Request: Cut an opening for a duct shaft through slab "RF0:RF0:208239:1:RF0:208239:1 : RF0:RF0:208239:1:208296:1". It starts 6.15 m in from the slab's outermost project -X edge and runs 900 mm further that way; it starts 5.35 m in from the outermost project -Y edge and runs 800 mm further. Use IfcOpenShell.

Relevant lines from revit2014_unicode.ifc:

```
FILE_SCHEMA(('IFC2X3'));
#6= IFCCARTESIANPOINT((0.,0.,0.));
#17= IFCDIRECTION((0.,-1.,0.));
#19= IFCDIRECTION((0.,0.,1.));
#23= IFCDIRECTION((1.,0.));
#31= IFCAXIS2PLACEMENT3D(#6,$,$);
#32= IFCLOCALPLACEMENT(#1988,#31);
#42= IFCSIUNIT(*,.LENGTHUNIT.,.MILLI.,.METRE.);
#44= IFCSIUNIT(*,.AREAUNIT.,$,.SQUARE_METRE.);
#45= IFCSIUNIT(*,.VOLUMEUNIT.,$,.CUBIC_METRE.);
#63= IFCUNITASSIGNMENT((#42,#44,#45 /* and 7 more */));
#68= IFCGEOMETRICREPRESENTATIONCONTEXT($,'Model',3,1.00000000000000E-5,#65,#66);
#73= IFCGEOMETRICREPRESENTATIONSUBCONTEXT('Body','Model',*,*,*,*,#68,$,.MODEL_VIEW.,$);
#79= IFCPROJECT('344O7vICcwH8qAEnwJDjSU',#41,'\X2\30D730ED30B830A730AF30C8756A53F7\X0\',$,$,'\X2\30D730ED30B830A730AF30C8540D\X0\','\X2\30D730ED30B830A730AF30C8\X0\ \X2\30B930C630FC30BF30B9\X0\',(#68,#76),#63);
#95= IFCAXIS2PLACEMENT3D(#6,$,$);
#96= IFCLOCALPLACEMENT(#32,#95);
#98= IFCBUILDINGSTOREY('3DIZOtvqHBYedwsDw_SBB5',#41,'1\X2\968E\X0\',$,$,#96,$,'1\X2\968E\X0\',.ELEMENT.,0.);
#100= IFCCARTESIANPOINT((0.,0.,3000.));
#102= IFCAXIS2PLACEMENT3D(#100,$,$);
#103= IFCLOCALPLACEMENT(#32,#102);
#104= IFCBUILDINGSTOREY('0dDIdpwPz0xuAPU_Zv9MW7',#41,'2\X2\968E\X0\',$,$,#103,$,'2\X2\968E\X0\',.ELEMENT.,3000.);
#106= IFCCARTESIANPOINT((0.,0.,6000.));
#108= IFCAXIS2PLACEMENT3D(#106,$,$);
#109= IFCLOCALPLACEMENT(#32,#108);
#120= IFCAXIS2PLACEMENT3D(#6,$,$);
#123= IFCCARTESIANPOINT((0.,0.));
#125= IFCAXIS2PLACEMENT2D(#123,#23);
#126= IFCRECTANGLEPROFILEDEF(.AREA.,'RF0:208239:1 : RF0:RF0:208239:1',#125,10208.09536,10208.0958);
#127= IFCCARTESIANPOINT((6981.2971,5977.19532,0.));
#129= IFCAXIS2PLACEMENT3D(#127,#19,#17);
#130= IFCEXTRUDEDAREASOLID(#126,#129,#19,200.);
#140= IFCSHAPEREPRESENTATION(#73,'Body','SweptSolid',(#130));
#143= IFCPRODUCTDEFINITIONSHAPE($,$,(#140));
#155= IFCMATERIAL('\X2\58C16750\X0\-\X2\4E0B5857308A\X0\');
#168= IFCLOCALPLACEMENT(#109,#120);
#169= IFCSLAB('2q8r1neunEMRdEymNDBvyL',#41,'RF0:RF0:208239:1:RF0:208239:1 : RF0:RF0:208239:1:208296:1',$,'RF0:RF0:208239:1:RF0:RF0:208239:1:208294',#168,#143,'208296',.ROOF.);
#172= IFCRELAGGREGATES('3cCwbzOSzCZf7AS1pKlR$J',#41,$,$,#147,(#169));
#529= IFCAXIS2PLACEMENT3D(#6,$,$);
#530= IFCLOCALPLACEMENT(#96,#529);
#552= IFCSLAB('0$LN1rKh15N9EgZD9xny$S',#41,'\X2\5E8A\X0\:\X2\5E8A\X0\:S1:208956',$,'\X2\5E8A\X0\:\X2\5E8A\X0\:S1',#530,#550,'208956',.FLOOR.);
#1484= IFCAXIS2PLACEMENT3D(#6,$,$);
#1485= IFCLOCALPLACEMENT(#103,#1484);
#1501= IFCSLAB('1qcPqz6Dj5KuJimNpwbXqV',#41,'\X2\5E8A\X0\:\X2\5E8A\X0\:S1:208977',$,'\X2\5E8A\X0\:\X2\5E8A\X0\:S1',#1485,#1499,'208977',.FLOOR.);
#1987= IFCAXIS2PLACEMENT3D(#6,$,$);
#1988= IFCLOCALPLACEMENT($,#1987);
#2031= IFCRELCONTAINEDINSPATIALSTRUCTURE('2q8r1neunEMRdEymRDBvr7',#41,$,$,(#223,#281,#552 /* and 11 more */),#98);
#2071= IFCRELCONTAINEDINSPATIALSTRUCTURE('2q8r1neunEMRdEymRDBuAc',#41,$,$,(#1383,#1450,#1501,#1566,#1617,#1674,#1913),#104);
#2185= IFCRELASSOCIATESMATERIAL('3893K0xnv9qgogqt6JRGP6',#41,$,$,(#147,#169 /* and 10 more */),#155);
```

```python
import numpy as np
import ifcopenshell
import ifcopenshell.api.feature
import ifcopenshell.api.geometry
import ifcopenshell.api.root
import ifcopenshell.geom
import ifcopenshell.util.placement
import ifcopenshell.util.representation
import ifcopenshell.util.shape
import ifcopenshell.util.unit

model = ifcopenshell.open("revit2014_unicode.ifc")
unit_scale = ifcopenshell.util.unit.calculate_unit_scale(model)
settings = ifcopenshell.geom.settings()


def volume(element):
    """Net volume in cubic metres, openings subtracted."""
    shape = ifcopenshell.geom.create_shape(settings, element)
    return ifcopenshell.util.shape.get_volume(shape.geometry)


slab = model.by_id(169)
before = volume(slab)

# Extent in the slab's own axes, in metres. The edges named are its -X and -Y sides.
slab_shape = ifcopenshell.geom.create_shape(settings, slab)
vertices = ifcopenshell.util.shape.get_vertices(slab_shape.geometry)
x_min, y_min, bottom = vertices.min(axis=0)
top = vertices[:, 2].max()

opening = ifcopenshell.api.root.create_entity(model, ifc_class="IfcOpeningElement", name="Duct shaft opening")
context = ifcopenshell.util.representation.get_context(model, "Model", "Body", "MODEL_VIEW")
width, depth = 0.9, 0.8
outline = [(0.0, 0.0), (width, 0.0), (width, depth), (0.0, depth), (0.0, 0.0)]
# Overshoot both faces by 50 mm so the cut is clean.
shape = ifcopenshell.api.geometry.add_slab_representation(
    model, context=context, depth=top - bottom + 0.1, polyline=outline
)
ifcopenshell.api.geometry.assign_representation(model, product=opening, representation=shape)

matrix = ifcopenshell.util.placement.get_local_placement(slab.ObjectPlacement)
matrix[:, 3] = matrix @ np.append(np.array([x_min + 6.15, y_min + 5.35, bottom - 0.05]) / unit_scale, 1.0)
ifcopenshell.api.geometry.edit_object_placement(model, product=opening, matrix=matrix, is_si=False)
ifcopenshell.api.feature.add_feature(model, feature=opening, element=slab)

after = volume(slab)

print(f"slab volume {before:.3f} -> {after:.3f} m3")

model.write("revit2014_unicode_updated.ifc")
```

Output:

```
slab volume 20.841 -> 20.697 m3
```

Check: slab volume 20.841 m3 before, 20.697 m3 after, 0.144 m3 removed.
